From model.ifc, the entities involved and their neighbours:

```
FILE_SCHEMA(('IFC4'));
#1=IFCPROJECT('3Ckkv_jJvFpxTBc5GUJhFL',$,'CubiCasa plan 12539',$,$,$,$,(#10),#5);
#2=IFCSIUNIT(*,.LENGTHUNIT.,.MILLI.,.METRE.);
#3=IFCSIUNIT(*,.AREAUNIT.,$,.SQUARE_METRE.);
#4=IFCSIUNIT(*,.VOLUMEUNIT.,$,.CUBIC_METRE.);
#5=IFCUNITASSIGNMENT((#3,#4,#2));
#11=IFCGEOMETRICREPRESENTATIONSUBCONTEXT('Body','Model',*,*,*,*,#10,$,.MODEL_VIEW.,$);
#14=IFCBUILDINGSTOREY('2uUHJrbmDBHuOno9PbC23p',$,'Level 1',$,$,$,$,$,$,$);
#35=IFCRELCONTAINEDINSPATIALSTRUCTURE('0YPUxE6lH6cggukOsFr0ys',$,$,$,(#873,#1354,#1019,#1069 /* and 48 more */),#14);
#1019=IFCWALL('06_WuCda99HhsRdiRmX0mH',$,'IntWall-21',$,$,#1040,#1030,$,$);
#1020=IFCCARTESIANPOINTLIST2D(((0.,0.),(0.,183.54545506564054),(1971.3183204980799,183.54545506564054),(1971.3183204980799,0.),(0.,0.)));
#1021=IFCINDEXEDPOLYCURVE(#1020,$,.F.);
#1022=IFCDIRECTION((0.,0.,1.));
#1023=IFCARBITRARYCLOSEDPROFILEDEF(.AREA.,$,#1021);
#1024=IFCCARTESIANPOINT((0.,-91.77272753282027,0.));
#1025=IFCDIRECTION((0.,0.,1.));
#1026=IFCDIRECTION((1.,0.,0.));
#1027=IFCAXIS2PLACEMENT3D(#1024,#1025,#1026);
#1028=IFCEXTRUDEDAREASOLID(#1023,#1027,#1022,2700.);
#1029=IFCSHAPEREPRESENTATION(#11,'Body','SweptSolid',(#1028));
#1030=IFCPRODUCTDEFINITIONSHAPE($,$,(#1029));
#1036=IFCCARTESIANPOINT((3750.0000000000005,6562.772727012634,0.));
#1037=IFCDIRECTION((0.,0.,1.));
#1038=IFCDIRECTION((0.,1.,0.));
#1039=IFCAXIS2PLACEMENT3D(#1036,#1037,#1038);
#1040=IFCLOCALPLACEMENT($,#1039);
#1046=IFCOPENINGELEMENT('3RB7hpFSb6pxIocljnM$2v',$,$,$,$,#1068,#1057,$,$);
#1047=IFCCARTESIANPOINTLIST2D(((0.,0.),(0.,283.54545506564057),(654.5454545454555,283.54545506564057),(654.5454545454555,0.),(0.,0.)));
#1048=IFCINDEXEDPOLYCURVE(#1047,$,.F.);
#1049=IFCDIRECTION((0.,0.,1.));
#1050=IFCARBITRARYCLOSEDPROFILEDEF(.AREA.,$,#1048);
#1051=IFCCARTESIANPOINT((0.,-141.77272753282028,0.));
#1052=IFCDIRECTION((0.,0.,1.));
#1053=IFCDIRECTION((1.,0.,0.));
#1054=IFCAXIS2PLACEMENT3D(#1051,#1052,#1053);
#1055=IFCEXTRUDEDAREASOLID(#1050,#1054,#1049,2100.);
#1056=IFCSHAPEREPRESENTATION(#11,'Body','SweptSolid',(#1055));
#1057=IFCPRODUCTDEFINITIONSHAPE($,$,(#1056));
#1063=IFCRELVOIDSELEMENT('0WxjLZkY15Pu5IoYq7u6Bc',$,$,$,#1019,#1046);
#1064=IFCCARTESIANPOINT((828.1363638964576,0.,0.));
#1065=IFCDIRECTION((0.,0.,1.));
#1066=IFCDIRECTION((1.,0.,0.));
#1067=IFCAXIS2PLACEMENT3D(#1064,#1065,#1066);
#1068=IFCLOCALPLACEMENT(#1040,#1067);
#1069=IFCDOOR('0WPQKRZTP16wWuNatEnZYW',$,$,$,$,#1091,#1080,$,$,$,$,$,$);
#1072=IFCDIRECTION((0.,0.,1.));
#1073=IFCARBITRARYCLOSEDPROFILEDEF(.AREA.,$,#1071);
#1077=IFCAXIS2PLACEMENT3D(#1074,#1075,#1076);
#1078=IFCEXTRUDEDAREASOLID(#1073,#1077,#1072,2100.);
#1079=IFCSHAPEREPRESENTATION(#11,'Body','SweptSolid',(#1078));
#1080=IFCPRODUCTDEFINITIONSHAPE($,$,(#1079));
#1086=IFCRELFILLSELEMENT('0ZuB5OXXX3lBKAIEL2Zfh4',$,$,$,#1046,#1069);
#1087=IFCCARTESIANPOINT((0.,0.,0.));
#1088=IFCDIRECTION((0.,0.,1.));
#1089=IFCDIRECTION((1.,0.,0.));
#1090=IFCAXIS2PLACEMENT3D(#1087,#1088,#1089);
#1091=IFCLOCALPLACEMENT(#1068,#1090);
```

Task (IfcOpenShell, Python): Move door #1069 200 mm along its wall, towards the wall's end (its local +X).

```python
import ifcopenshell
import ifcopenshell.api.geometry
import ifcopenshell.util.placement

model = ifcopenshell.open("model.ifc")

door = model.by_guid("0WPQKRZTP16wWuNatEnZYW")
opening = door.FillsVoids[0].RelatingOpeningElement
wall = opening.VoidsElements[0].RelatingBuildingElement

wall_matrix = ifcopenshell.util.placement.get_local_placement(wall.ObjectPlacement)
shift = wall_matrix[:3, 0] * 200.0
before = ifcopenshell.util.placement.get_local_placement(door.ObjectPlacement)[:3, 3].copy()

# The door is placed relative to its opening, so it follows when the opening moves.
matrix = ifcopenshell.util.placement.get_local_placement(opening.ObjectPlacement)
matrix[:3, 3] += shift
ifcopenshell.api.geometry.edit_object_placement(
    model, product=opening, matrix=matrix, is_si=False, should_transform_children=True
)

after = ifcopenshell.util.placement.get_local_placement(door.ObjectPlacement)[:3, 3]
print("door moved by", (after - before).round(3) + 0.0)

model.write("model_edited.ifc")
```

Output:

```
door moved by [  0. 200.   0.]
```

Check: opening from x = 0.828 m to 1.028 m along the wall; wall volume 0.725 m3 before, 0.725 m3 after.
